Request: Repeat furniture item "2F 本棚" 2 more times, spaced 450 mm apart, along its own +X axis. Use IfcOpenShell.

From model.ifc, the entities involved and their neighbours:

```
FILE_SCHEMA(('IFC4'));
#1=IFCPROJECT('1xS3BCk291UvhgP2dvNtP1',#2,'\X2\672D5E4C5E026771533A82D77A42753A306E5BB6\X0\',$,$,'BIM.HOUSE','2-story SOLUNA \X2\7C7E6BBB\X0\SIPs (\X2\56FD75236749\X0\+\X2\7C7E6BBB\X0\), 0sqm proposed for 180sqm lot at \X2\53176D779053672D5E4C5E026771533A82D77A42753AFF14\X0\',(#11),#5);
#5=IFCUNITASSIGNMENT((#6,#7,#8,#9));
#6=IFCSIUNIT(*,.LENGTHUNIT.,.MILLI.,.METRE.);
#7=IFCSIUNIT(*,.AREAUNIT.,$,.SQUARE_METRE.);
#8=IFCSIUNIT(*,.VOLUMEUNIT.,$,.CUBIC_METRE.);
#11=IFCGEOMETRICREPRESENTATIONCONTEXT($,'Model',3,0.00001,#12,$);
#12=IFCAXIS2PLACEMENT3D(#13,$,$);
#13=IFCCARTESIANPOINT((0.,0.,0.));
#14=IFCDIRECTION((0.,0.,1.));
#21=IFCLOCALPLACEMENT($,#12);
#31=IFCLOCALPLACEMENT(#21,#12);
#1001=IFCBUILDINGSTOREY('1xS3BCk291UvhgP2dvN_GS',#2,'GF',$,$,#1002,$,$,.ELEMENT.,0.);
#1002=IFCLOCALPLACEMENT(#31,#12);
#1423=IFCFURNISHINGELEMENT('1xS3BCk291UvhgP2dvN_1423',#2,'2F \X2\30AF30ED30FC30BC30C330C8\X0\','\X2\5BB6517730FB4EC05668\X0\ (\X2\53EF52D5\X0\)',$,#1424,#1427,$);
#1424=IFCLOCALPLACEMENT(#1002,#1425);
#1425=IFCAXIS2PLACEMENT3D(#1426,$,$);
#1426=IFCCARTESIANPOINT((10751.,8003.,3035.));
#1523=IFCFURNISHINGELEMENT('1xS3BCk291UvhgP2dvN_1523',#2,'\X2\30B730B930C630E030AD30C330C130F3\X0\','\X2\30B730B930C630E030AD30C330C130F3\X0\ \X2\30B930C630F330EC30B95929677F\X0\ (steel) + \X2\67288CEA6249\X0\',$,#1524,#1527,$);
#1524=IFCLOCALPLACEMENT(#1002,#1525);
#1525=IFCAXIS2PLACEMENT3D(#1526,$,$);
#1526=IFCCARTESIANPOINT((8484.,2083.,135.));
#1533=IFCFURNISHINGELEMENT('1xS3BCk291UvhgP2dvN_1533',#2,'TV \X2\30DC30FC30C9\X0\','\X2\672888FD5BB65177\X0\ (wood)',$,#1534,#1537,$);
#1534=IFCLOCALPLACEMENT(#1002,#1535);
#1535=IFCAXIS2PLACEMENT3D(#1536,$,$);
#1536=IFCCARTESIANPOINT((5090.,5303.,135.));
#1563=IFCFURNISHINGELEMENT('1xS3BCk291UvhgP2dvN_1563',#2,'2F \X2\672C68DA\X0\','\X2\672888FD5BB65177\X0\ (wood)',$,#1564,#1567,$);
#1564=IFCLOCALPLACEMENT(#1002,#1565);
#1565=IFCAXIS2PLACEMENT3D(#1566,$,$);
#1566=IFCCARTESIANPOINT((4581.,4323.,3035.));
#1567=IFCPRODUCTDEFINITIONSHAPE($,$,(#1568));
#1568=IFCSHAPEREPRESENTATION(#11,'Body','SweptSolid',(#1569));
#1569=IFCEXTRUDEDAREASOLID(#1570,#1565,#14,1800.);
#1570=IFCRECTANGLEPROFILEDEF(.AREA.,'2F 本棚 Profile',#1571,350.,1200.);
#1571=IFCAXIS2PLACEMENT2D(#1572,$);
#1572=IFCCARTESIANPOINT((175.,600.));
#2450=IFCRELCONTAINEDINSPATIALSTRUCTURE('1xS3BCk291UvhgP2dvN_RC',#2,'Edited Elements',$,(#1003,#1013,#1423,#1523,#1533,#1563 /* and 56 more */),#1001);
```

```python
import ifcopenshell
import ifcopenshell.api.geometry
import ifcopenshell.api.root
import ifcopenshell.util.element
import ifcopenshell.util.placement
import ifcopenshell.util.unit

model = ifcopenshell.open("model.ifc")
unit_scale = ifcopenshell.util.unit.calculate_unit_scale(model)


def reuse_history(source, copy):
    """copy_class also copies each property set's owner history, people and application; keep the originals."""
    for rel in copy.IsDefinedBy:
        if rel.is_a("IfcRelDefinesByProperties") and (history := rel.RelatingPropertyDefinition.OwnerHistory):
            rel.RelatingPropertyDefinition.OwnerHistory = source.OwnerHistory
            ifcopenshell.util.element.remove_deep2(model, history)


source = model.by_id(1563)
base = ifcopenshell.util.placement.get_local_placement(source.ObjectPlacement)
step = base[:3, 0] * 0.45 / unit_scale

for i in range(1, 3):
    copy = ifcopenshell.api.root.copy_class(model, product=source)
    copy.Representation = ifcopenshell.util.element.copy_deep(
        model, source.Representation, exclude=["IfcGeometricRepresentationContext", "IfcRepresentationMap"]
    )
    reuse_history(source, copy)
    matrix = base.copy()
    matrix[:3, 3] += i * step
    print("added at", matrix[:3, 3].round(3) + 0.0)
    ifcopenshell.api.geometry.edit_object_placement(model, product=copy, matrix=matrix, is_si=False)

model.write("model_updated.ifc")
```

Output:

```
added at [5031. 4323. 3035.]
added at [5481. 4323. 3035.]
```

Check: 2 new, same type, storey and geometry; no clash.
